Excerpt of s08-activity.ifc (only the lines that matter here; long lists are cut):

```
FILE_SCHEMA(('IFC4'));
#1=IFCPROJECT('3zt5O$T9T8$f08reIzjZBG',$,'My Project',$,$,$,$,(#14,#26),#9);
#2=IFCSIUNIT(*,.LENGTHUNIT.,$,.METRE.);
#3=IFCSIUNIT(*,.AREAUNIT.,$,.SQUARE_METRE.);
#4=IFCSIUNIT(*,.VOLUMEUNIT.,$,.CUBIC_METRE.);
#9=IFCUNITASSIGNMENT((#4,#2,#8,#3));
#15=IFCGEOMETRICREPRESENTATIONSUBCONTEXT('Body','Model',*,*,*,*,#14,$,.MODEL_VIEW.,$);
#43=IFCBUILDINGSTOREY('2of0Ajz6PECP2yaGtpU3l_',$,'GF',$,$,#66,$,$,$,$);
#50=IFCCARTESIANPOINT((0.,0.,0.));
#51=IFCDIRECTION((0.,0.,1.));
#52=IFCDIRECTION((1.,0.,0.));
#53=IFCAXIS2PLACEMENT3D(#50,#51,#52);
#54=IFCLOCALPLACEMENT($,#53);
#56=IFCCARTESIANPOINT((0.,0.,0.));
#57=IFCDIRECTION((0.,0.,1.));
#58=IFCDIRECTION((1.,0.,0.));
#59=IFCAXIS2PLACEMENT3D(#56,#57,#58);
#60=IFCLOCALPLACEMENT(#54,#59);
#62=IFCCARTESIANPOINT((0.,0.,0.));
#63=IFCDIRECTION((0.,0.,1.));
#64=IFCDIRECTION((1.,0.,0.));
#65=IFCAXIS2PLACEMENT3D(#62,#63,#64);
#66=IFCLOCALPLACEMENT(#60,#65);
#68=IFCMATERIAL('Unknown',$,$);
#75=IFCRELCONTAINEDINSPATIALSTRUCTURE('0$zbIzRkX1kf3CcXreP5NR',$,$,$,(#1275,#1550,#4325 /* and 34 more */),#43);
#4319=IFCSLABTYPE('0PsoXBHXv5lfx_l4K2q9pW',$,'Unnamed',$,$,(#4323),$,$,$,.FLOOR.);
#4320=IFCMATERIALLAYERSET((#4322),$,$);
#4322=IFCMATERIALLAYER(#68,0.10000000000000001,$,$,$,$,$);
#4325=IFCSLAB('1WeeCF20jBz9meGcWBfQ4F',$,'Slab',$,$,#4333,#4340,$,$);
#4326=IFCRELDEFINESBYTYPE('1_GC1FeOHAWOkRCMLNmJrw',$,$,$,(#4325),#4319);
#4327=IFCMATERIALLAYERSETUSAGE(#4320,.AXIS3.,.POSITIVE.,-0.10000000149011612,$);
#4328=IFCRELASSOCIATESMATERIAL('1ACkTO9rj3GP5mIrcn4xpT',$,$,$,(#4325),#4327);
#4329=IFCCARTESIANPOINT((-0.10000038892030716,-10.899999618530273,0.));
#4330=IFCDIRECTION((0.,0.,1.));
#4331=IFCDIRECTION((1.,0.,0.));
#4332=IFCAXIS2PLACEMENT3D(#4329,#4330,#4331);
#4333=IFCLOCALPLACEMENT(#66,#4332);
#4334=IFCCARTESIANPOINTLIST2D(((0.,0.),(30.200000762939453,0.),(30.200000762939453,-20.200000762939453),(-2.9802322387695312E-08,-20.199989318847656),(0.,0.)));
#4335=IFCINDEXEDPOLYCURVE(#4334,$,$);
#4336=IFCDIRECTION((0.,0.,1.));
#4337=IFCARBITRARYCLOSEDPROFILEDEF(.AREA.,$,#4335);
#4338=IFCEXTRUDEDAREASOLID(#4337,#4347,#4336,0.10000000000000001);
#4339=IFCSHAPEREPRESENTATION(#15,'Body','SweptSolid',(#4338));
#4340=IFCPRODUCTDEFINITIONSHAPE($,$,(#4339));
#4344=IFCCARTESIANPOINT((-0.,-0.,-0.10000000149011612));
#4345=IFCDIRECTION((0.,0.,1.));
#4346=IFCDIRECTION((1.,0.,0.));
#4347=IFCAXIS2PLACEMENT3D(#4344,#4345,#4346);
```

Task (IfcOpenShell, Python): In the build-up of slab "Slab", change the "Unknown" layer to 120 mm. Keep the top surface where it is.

```python
import ifcopenshell
import ifcopenshell.util.element
import ifcopenshell.util.representation
import ifcopenshell.util.unit

model = ifcopenshell.open("s08-activity.ifc")
unit_scale = ifcopenshell.util.unit.calculate_unit_scale(model)

layer_set = model.by_id(4320)
layer = next(l for l in layer_set.MaterialLayers if l.Material and l.Material.Name == "Unknown")
change = 0.12 / unit_scale - layer.LayerThickness
layer.LayerThickness += change

# Geometry does not follow the layer set by itself.
slabs = [e for e in ifcopenshell.util.element.get_elements_by_material(model, layer_set) if e.is_a("IfcSlab")]
for slab in sorted(slabs, key=lambda e: e.id()):
    body = ifcopenshell.util.representation.get_representation(slab, "Model", "Body")
    solid = body.Items[0]
    old_depth = solid.Depth
    solid.Depth += change
    # Extruded upwards: lower the start of the extrusion so the top stays.
    x, y, z = solid.Position.Location.Coordinates
    solid.Position.Location = model.createIfcCartesianPoint((x, y, z - change))
    print(slab.id(), f"{old_depth:g} -> {solid.Depth:g}")

# The layers are counted up from the underside, which has moved.
for usage in {ifcopenshell.util.element.get_material(slab) for slab in slabs}:
    usage.OffsetFromReferenceLine -= change

model.write("s08-activity_edited.ifc")
```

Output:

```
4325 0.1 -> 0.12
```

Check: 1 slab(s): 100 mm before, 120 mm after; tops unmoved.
